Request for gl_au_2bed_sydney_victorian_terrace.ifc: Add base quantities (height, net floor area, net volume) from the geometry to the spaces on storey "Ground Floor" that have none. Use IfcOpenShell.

First a look at what the model holds.

```python
import ifcopenshell
import ifcopenshell.util.element
import ifcopenshell.util.unit

model = ifcopenshell.open("gl_au_2bed_sydney_victorian_terrace.ifc")
print(model.schema)
for unit_type in ("LENGTHUNIT", "AREAUNIT", "VOLUMEUNIT"):
    print(unit_type, ifcopenshell.util.unit.calculate_unit_scale(model, unit_type))
storey = next(s for s in model.by_type("IfcBuildingStorey") if s.Name == "Ground Floor")
spaces = [e for e in ifcopenshell.util.element.get_decomposition(storey) if e.is_a("IfcSpace")]
for e in sorted(spaces, key=lambda e: e.id()):
    print(e.id(), e.is_a(), e.Name, list(ifcopenshell.util.element.get_psets(e, qtos_only=True)), sep=" | ")
```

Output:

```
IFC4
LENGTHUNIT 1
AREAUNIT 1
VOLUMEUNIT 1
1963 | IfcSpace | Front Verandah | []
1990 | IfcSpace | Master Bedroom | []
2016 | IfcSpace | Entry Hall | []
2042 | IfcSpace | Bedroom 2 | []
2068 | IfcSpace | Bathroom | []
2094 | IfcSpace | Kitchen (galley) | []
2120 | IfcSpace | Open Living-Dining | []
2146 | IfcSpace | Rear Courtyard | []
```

```python
import ifcopenshell
import ifcopenshell.api.pset
import ifcopenshell.geom
import ifcopenshell.util.element
import ifcopenshell.util.shape
import ifcopenshell.util.unit

model = ifcopenshell.open("gl_au_2bed_sydney_victorian_terrace.ifc")
unit_scale = ifcopenshell.util.unit.calculate_unit_scale(model)
area_scale = ifcopenshell.util.unit.calculate_unit_scale(model, "AREAUNIT")
volume_scale = ifcopenshell.util.unit.calculate_unit_scale(model, "VOLUMEUNIT")
settings = ifcopenshell.geom.settings()

storey = next(s for s in model.by_type("IfcBuildingStorey") if s.Name == "Ground Floor")
spaces = [e for e in ifcopenshell.util.element.get_decomposition(storey) if e.is_a("IfcSpace")]

for e in sorted(spaces, key=lambda e: e.id()):
    if ifcopenshell.util.element.get_psets(e, qtos_only=True, should_inherit=False):
        continue
    # Geometry comes back in metres, in the element's own axes.
    shape = ifcopenshell.geom.create_shape(settings, e)
    values = {
        "Height": ifcopenshell.util.shape.get_z(shape.geometry) / unit_scale,
        "NetFloorArea": ifcopenshell.util.shape.get_footprint_area(shape.geometry) / area_scale,
        "NetVolume": ifcopenshell.util.shape.get_volume(shape.geometry) / volume_scale,
    }
    qto = ifcopenshell.api.pset.add_qto(model, product=e, name="Qto_SpaceBaseQuantities")
    ifcopenshell.api.pset.edit_qto(model, qto=qto, properties=values)
    print(e.id(), {k: round(v, 3) for k, v in values.items()})

model.write("gl_au_2bed_sydney_victorian_terrace-out.ifc")
```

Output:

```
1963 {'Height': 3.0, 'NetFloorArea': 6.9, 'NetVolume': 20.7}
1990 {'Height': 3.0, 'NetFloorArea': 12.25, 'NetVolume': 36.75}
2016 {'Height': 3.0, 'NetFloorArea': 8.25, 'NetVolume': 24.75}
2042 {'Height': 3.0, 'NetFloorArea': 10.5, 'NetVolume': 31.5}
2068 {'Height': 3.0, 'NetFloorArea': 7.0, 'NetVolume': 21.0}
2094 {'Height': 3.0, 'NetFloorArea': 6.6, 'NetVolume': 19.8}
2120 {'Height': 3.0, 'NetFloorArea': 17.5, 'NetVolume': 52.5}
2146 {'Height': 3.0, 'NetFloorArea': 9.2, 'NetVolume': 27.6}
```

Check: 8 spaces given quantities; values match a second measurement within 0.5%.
